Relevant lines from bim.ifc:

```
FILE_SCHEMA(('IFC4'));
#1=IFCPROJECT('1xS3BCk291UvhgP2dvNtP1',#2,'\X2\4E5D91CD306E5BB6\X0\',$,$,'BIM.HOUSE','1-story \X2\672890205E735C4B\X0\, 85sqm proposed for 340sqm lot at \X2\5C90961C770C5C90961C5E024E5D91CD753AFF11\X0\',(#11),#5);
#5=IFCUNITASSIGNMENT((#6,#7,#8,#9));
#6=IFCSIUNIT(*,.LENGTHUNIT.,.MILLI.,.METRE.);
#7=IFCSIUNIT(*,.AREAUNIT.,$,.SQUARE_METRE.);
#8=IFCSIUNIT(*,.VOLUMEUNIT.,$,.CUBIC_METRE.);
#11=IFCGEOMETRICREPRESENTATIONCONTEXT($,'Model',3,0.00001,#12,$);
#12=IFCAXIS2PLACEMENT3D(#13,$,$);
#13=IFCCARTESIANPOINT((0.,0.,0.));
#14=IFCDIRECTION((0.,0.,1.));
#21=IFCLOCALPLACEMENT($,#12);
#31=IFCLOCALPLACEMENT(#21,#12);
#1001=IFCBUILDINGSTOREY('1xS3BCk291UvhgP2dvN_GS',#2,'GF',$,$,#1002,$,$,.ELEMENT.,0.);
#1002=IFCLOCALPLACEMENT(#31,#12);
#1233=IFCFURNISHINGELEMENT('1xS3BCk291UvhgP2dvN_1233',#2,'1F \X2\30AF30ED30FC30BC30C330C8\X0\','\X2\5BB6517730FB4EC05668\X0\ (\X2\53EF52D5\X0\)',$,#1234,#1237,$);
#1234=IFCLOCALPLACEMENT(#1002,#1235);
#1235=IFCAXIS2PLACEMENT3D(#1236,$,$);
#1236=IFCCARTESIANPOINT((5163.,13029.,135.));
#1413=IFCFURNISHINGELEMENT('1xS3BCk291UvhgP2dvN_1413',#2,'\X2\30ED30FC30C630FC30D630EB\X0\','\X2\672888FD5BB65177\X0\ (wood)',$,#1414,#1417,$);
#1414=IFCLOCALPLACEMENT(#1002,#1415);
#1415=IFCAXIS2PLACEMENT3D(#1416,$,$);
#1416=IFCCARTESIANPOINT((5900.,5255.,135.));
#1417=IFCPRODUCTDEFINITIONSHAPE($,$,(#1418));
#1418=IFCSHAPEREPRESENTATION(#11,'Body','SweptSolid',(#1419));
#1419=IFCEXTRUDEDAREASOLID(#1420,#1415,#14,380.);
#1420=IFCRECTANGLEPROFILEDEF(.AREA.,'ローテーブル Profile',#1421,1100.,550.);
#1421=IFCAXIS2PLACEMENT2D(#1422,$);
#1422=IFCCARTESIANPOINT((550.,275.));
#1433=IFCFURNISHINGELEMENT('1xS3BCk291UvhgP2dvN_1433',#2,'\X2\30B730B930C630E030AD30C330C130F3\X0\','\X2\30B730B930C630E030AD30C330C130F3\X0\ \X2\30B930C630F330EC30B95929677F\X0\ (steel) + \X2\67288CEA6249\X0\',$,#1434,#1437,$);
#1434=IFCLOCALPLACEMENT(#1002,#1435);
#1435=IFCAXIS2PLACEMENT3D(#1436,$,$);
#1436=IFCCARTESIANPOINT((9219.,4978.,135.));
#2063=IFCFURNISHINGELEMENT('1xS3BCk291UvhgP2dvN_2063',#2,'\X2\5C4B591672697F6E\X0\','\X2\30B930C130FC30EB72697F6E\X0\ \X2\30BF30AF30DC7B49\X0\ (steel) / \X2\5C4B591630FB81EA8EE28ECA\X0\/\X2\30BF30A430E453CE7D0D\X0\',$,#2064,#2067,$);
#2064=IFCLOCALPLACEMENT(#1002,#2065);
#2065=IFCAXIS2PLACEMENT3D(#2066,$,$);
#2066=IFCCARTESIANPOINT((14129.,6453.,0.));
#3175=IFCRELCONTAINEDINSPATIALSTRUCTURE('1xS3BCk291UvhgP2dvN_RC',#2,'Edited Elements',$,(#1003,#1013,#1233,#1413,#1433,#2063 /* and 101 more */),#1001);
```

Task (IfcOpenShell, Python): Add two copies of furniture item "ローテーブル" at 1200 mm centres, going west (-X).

```python
import numpy as np
import ifcopenshell
import ifcopenshell.api.geometry
import ifcopenshell.api.root
import ifcopenshell.util.element
import ifcopenshell.util.placement
import ifcopenshell.util.unit

model = ifcopenshell.open("bim.ifc")
unit_scale = ifcopenshell.util.unit.calculate_unit_scale(model)


def reuse_history(source, copy):
    """copy_class also copies each property set's owner history, people and application; keep the originals."""
    for rel in copy.IsDefinedBy:
        if rel.is_a("IfcRelDefinesByProperties") and (history := rel.RelatingPropertyDefinition.OwnerHistory):
            rel.RelatingPropertyDefinition.OwnerHistory = source.OwnerHistory
            ifcopenshell.util.element.remove_deep2(model, history)


source = model.by_id(1413)
base = ifcopenshell.util.placement.get_local_placement(source.ObjectPlacement)
step = np.array([-1.0, 0.0, 0.0]) * 1.2 / unit_scale

for i in range(1, 3):
    copy = ifcopenshell.api.root.copy_class(model, product=source)
    copy.Representation = ifcopenshell.util.element.copy_deep(
        model, source.Representation, exclude=["IfcGeometricRepresentationContext", "IfcRepresentationMap"]
    )
    reuse_history(source, copy)
    matrix = base.copy()
    matrix[:3, 3] += i * step
    print("added at", matrix[:3, 3].round(3) + 0.0)
    ifcopenshell.api.geometry.edit_object_placement(model, product=copy, matrix=matrix, is_si=False)

model.write("bim-out.ifc")
```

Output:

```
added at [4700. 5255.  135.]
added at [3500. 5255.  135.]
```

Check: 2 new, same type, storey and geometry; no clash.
